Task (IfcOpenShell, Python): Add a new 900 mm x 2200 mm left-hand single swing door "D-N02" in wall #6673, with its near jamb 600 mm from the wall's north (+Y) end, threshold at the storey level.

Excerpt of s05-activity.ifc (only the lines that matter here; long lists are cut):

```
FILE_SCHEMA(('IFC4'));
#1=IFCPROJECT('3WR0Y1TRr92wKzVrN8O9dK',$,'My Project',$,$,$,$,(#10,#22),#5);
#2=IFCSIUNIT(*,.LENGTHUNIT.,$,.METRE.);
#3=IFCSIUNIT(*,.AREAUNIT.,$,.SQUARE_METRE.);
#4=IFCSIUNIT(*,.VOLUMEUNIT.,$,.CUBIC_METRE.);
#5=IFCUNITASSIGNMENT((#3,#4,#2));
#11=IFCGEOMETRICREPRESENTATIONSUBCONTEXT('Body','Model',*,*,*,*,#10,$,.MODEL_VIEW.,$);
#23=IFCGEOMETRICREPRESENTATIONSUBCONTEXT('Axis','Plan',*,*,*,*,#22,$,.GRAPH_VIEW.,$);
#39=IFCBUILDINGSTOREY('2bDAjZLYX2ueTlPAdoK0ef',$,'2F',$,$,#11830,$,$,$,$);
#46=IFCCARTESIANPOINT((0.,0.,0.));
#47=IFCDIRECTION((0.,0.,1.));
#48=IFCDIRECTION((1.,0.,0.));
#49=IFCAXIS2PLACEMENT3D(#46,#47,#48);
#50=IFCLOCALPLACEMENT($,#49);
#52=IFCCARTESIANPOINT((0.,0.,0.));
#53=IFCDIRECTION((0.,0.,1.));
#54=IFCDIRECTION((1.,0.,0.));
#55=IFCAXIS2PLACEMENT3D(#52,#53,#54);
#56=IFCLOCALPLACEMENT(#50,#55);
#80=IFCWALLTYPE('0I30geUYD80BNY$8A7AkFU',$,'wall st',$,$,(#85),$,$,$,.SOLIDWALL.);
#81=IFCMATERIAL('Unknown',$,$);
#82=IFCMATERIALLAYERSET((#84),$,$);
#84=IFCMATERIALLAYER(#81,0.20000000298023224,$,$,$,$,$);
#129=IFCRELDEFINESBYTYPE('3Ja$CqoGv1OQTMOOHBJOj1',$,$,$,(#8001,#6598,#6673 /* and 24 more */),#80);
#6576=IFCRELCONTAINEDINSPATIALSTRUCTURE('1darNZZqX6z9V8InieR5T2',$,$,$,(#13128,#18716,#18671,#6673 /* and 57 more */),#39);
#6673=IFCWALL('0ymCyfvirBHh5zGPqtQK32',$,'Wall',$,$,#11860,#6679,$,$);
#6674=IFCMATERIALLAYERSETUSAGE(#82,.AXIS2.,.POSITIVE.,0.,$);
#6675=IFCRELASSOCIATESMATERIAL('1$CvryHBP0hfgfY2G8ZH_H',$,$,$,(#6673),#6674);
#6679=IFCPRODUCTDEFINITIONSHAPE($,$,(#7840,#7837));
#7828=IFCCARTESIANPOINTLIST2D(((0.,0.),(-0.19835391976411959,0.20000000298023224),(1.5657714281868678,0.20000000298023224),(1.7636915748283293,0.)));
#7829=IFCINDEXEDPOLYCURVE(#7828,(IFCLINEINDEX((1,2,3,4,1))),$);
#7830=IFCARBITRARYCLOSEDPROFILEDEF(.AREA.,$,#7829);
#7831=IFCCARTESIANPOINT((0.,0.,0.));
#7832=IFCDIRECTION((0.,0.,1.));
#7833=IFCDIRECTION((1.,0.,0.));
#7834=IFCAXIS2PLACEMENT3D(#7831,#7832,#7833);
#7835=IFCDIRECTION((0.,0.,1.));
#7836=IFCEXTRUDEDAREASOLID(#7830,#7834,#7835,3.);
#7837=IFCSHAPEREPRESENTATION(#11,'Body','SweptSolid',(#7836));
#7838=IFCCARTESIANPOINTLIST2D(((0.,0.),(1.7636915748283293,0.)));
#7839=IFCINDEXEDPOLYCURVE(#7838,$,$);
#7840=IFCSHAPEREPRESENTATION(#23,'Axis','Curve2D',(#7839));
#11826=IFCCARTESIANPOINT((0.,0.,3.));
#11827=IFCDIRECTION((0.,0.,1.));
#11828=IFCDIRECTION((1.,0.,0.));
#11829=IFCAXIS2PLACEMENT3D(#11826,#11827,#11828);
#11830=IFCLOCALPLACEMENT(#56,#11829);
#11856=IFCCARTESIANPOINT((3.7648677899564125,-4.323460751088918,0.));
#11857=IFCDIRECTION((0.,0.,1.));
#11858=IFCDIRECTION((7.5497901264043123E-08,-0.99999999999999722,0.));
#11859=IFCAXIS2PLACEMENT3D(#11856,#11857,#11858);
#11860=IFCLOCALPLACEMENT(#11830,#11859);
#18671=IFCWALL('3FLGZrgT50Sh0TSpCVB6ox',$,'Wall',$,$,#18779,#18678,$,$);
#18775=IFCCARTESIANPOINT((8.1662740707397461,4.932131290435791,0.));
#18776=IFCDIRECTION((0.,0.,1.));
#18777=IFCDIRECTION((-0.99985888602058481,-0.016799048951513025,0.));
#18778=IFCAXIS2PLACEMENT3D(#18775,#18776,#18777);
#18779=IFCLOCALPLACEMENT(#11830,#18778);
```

```python
import numpy as np
import ifcopenshell
import ifcopenshell.api.feature
import ifcopenshell.api.geometry
import ifcopenshell.api.root
import ifcopenshell.api.spatial
import ifcopenshell.geom
import ifcopenshell.util.element
import ifcopenshell.util.placement
import ifcopenshell.util.representation
import ifcopenshell.util.shape
import ifcopenshell.util.unit

model = ifcopenshell.open("s05-activity.ifc")
unit_scale = ifcopenshell.util.unit.calculate_unit_scale(model)
settings = ifcopenshell.geom.settings()


def volume(element):
    """Net volume in cubic metres, openings subtracted."""
    shape = ifcopenshell.geom.create_shape(settings, element)
    return ifcopenshell.util.shape.get_volume(shape.geometry)


wall = model.by_guid("0ymCyfvirBHh5zGPqtQK32")
storey = ifcopenshell.util.element.get_container(wall, ifc_class="IfcBuildingStorey")
context = ifcopenshell.util.representation.get_context(model, "Model", "Body", "MODEL_VIEW")
before = volume(wall)

width, height, from_end, sill = 0.9, 2.2, 0.6, 0.0  # metres

# The wall runs along its own X axis, and the end named is its -X end.
wall_shape = ifcopenshell.geom.create_shape(settings, wall)
x, y, z = ifcopenshell.util.shape.get_vertices(wall_shape.geometry).T
start = x.min() + from_end
face, thickness = float(y.min()), float(y.max() - y.min())
wall_matrix = ifcopenshell.util.placement.get_local_placement(wall.ObjectPlacement)
level = ifcopenshell.util.placement.get_local_placement(storey.ObjectPlacement)[2, 3]


def in_wall(x, y):
    """Placement at x, y metres in the wall's axes, at sill height."""
    matrix = wall_matrix.copy()
    matrix[:, 3] = wall_matrix @ np.array([x / unit_scale, y / unit_scale, 0.0, 1.0])
    matrix[2, 3] = level + sill / unit_scale
    return matrix


# Opening: a box that overshoots both wall faces by 50 mm.
opening = ifcopenshell.api.root.create_entity(model, ifc_class="IfcOpeningElement", predefined_type="OPENING")
box = ifcopenshell.api.geometry.add_wall_representation(
    model, context=context, length=width, height=height, thickness=thickness + 0.1
)
ifcopenshell.api.geometry.assign_representation(model, product=opening, representation=box)
ifcopenshell.api.geometry.edit_object_placement(model, product=opening, matrix=in_wall(start, face - 0.05), is_si=False)
ifcopenshell.api.feature.add_feature(model, feature=opening, element=wall)

door = ifcopenshell.api.root.create_entity(model, ifc_class="IfcDoor", name="D-N02", predefined_type="DOOR")
door.OverallWidth, door.OverallHeight = width / unit_scale, height / unit_scale
door.OperationType = "SINGLE_SWING_LEFT"
body = ifcopenshell.api.geometry.add_door_representation(
    model,
    context=context,
    overall_width=door.OverallWidth,
    overall_height=door.OverallHeight,
    operation_type="SINGLE_SWING_LEFT",
    lining_properties={"LiningDepth": thickness / unit_scale, "ThresholdDepth": thickness / unit_scale},
)
ifcopenshell.api.geometry.assign_representation(model, product=door, representation=body)
ifcopenshell.api.spatial.assign_container(model, products=[door], relating_structure=storey)
ifcopenshell.api.feature.add_filling(model, opening=opening, element=door)

# The lining spans the wall, so the door starts at the wall face.
ifcopenshell.api.geometry.edit_object_placement(model, product=door, matrix=in_wall(start, face), is_si=False)

after = volume(wall)

print(f"wall volume {before:.3f} -> {after:.3f} m3")

model.write("s05-activity-out.ifc")
```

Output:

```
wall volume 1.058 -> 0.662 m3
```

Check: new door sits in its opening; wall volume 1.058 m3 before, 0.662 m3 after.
